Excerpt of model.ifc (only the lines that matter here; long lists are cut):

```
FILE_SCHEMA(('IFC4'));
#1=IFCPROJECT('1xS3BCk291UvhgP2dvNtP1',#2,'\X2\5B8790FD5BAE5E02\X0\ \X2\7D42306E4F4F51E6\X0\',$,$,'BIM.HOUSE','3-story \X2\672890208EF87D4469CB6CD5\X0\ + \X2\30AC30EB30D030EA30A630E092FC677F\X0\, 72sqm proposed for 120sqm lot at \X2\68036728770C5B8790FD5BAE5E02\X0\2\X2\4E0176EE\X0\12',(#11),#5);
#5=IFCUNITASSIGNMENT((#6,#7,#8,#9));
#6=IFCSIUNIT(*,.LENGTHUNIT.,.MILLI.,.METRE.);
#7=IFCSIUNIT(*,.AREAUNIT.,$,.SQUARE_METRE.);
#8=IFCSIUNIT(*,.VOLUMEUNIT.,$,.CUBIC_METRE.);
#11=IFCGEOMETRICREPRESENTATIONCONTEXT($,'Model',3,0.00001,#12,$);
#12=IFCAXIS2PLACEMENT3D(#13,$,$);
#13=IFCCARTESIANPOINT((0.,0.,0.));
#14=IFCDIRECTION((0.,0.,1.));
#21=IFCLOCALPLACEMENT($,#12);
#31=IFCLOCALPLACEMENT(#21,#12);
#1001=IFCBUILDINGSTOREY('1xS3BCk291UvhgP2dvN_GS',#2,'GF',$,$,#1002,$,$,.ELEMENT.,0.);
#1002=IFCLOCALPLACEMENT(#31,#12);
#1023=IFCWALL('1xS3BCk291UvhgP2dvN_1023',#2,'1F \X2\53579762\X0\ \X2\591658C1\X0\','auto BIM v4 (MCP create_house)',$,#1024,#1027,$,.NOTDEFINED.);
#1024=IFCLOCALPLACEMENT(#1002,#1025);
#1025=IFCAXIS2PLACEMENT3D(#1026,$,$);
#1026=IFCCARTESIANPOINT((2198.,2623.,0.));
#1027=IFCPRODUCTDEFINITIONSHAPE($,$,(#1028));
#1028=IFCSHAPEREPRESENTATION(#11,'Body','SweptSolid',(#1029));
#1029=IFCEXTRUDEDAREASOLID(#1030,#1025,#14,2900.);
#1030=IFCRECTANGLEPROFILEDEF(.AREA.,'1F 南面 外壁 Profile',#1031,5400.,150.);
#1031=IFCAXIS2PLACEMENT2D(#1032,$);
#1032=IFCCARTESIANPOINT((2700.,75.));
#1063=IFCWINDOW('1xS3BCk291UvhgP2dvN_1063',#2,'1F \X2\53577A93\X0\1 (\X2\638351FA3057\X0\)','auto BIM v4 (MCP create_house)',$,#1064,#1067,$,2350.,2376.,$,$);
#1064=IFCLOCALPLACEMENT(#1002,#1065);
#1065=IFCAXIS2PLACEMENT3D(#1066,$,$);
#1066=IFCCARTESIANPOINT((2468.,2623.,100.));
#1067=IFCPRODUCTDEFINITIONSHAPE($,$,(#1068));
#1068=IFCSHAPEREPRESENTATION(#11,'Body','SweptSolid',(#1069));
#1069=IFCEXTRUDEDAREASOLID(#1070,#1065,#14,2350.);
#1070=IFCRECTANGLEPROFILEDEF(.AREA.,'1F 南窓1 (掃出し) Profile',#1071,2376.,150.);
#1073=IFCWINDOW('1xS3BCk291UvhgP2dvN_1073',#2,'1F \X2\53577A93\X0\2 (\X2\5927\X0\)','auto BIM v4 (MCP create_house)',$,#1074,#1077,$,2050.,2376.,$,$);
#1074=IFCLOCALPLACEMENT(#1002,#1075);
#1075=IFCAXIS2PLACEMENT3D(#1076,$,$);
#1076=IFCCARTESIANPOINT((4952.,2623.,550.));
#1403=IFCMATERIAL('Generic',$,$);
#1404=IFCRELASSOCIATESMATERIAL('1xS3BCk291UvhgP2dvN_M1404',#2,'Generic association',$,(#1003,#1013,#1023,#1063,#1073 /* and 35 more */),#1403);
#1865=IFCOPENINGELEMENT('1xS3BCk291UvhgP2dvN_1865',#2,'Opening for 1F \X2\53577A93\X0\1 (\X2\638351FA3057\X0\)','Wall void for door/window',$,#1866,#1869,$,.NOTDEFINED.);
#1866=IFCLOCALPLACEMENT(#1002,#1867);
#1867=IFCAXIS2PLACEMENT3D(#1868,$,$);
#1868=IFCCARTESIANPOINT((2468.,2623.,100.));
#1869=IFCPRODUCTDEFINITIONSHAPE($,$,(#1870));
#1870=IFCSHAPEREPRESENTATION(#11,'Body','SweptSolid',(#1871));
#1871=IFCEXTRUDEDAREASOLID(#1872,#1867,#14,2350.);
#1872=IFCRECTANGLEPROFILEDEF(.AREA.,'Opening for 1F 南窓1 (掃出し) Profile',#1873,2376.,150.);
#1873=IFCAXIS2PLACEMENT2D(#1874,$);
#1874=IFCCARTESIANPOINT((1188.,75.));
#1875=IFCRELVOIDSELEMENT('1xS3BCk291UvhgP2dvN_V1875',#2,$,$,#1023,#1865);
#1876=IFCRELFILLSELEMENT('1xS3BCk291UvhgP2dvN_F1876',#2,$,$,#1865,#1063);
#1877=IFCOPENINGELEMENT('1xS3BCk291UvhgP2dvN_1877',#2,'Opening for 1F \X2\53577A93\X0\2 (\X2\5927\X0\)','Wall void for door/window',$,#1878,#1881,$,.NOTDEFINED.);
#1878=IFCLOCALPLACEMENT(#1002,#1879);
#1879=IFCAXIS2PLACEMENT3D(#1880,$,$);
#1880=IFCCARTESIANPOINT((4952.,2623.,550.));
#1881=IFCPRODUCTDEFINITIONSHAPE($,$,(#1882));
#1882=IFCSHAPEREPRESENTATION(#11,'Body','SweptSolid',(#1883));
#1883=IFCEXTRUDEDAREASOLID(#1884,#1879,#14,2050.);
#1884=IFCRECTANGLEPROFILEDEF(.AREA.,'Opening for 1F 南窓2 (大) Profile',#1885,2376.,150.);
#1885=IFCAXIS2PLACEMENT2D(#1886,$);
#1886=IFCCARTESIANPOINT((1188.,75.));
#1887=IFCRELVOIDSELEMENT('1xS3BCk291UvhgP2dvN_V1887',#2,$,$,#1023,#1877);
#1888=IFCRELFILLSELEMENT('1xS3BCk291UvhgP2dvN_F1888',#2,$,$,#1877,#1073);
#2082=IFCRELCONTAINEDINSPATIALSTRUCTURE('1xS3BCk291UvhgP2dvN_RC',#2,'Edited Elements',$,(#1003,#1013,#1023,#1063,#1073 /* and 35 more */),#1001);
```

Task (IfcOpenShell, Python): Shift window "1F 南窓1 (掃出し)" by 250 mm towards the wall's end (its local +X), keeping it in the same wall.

```python
import ifcopenshell
import ifcopenshell.api.geometry
import ifcopenshell.util.placement
import ifcopenshell.util.unit

model = ifcopenshell.open("model.ifc")
unit_scale = ifcopenshell.util.unit.calculate_unit_scale(model)

window = model.by_guid("1xS3BCk291UvhgP2dvN_1063")
opening = window.FillsVoids[0].RelatingOpeningElement
wall = opening.VoidsElements[0].RelatingBuildingElement

wall_matrix = ifcopenshell.util.placement.get_local_placement(wall.ObjectPlacement)
shift = wall_matrix[:3, 0] * 0.25 / unit_scale
before = ifcopenshell.util.placement.get_local_placement(window.ObjectPlacement)[:3, 3].copy()

# The window is not placed relative to its opening, so move both.
for product in (opening, window):
    matrix = ifcopenshell.util.placement.get_local_placement(product.ObjectPlacement)
    matrix[:3, 3] += shift
    ifcopenshell.api.geometry.edit_object_placement(model, product=product, matrix=matrix, is_si=False)

after = ifcopenshell.util.placement.get_local_placement(window.ObjectPlacement)[:3, 3]
print("window moved by", (after - before).round(3) + 0.0)

model.write("model_updated.ifc")
```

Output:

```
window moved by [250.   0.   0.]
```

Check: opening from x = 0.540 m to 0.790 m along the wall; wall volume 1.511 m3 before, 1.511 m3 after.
